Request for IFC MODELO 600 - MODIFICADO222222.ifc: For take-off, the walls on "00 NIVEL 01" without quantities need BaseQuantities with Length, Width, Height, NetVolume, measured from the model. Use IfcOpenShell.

First a look at what the model holds.

```python
import ifcopenshell
import ifcopenshell.util.element
import ifcopenshell.util.unit

model = ifcopenshell.open("IFC MODELO 600 - MODIFICADO222222.ifc")
print(model.schema)
for unit_type in ("LENGTHUNIT", "AREAUNIT", "VOLUMEUNIT"):
    print(unit_type, ifcopenshell.util.unit.calculate_unit_scale(model, unit_type))
storey = next(s for s in model.by_type("IfcBuildingStorey") if s.Name == "00 NIVEL 01")
walls = [e for e in ifcopenshell.util.element.get_decomposition(storey) if e.is_a("IfcWall")]
for e in sorted(walls, key=lambda e: e.id()):
    print(e.id(), e.is_a(), e.Name, list(ifcopenshell.util.element.get_psets(e, qtos_only=True)), sep=" | ")
```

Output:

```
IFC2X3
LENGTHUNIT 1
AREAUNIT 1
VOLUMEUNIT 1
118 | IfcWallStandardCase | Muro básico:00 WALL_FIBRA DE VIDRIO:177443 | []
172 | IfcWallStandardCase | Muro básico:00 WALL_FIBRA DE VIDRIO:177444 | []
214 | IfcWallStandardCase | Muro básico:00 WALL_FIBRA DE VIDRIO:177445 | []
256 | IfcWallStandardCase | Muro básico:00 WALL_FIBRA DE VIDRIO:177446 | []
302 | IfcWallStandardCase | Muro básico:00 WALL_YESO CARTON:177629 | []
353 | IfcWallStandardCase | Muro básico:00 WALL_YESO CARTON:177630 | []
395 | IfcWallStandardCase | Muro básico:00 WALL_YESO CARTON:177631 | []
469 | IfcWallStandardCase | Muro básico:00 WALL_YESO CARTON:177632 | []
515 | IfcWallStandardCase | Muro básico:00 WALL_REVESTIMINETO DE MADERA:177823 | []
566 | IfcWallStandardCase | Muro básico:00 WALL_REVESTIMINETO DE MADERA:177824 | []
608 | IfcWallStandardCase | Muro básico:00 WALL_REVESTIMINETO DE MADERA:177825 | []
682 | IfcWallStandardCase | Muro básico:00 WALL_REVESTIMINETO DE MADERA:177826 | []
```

```python
import ifcopenshell
import ifcopenshell.api.pset
import ifcopenshell.geom
import ifcopenshell.util.element
import ifcopenshell.util.shape
import ifcopenshell.util.unit

model = ifcopenshell.open("IFC MODELO 600 - MODIFICADO222222.ifc")
unit_scale = ifcopenshell.util.unit.calculate_unit_scale(model)
volume_scale = ifcopenshell.util.unit.calculate_unit_scale(model, "VOLUMEUNIT")
settings = ifcopenshell.geom.settings()

storey = next(s for s in model.by_type("IfcBuildingStorey") if s.Name == "00 NIVEL 01")
walls = [e for e in ifcopenshell.util.element.get_decomposition(storey) if e.is_a("IfcWall")]

for e in sorted(walls, key=lambda e: e.id()):
    if ifcopenshell.util.element.get_psets(e, qtos_only=True, should_inherit=False):
        continue
    # Geometry comes back in metres, in the element's own axes.
    shape = ifcopenshell.geom.create_shape(settings, e)
    values = {
        "Length": ifcopenshell.util.shape.get_x(shape.geometry) / unit_scale,
        "Width": ifcopenshell.util.shape.get_y(shape.geometry) / unit_scale,
        "Height": ifcopenshell.util.shape.get_z(shape.geometry) / unit_scale,
        "NetVolume": ifcopenshell.util.shape.get_volume(shape.geometry) / volume_scale,
    }
    qto = ifcopenshell.api.pset.add_qto(model, product=e, name="BaseQuantities")
    ifcopenshell.api.pset.edit_qto(model, qto=qto, properties=values)
    print(e.id(), {k: round(v, 3) for k, v in values.items()})

model.write("IFC MODELO 600 - MODIFICADO222222_v2.ifc")
```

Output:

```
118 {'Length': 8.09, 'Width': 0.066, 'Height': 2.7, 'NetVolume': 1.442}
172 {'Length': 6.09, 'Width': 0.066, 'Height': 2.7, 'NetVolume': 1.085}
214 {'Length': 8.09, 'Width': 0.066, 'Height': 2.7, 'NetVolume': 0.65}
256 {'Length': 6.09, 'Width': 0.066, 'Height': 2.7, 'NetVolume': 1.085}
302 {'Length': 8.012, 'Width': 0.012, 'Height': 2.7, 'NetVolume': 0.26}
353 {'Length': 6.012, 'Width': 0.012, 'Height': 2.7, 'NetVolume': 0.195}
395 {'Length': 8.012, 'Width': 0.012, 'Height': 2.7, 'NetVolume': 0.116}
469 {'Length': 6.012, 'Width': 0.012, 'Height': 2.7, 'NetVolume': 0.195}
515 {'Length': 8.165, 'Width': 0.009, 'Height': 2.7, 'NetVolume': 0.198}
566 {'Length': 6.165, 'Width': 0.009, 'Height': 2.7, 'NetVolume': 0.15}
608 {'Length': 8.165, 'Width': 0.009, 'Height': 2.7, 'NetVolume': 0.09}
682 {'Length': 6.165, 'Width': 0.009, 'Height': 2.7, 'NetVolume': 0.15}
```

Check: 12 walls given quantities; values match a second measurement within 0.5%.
